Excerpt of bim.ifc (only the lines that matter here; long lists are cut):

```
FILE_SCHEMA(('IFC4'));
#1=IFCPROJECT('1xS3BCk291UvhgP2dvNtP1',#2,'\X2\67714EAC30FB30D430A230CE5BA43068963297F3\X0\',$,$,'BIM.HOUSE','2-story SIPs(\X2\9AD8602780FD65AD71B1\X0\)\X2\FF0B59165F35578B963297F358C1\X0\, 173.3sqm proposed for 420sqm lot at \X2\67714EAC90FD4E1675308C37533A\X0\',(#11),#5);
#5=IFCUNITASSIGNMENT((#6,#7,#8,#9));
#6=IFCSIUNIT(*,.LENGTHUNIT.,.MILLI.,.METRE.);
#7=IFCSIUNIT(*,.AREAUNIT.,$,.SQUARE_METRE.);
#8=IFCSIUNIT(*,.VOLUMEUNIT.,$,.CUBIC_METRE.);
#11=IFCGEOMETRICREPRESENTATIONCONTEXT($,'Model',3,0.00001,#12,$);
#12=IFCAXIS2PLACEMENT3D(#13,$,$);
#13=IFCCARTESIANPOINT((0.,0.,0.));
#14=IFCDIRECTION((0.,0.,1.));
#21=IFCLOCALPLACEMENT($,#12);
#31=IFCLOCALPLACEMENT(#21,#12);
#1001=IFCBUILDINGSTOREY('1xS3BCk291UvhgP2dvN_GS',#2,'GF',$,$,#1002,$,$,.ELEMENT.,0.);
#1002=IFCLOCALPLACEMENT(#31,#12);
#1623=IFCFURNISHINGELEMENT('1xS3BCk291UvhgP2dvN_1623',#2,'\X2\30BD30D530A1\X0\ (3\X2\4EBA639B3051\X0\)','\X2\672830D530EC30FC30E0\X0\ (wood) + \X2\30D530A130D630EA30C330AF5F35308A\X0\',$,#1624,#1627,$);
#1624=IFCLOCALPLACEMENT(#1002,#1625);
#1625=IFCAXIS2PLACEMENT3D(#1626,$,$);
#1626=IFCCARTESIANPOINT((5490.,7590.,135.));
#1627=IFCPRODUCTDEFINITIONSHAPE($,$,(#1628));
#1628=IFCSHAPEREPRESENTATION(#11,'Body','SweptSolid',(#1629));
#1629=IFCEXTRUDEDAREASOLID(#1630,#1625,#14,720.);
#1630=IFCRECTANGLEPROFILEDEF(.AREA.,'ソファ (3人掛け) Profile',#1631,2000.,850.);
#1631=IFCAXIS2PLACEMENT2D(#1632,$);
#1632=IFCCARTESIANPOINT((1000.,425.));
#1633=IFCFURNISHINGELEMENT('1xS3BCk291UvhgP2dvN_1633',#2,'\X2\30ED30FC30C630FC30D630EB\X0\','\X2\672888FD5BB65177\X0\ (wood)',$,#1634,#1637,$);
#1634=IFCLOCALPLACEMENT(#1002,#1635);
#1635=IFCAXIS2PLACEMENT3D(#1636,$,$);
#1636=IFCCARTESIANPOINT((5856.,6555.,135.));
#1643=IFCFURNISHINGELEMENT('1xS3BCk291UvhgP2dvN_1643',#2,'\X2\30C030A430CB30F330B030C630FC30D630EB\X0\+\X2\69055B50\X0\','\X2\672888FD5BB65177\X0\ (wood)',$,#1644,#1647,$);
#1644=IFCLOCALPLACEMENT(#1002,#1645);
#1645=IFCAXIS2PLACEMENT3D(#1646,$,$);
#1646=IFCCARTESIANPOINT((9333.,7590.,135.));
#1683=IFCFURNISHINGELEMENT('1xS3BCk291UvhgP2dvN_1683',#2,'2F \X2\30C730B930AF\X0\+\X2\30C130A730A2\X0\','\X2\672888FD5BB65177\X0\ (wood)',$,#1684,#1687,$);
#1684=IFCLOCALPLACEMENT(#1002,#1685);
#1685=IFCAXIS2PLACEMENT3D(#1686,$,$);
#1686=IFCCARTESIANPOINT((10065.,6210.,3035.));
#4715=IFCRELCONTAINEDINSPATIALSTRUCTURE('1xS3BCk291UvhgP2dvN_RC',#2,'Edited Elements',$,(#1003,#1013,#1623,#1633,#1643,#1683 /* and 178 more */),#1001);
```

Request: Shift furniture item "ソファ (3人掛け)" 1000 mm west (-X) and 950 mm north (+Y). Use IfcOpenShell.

```python
import ifcopenshell
import ifcopenshell.api.geometry
import ifcopenshell.util.placement
import ifcopenshell.util.unit

model = ifcopenshell.open("bim.ifc")
unit_scale = ifcopenshell.util.unit.calculate_unit_scale(model)

item = model.by_id(1623)
matrix = ifcopenshell.util.placement.get_local_placement(item.ObjectPlacement)
matrix[0, 3] -= 1 / unit_scale
matrix[1, 3] += 0.95 / unit_scale
ifcopenshell.api.geometry.edit_object_placement(model, product=item, matrix=matrix, is_si=False)

print(ifcopenshell.util.placement.get_local_placement(item.ObjectPlacement).round(3) + 0.0)

model.write("bim-out.ifc")
```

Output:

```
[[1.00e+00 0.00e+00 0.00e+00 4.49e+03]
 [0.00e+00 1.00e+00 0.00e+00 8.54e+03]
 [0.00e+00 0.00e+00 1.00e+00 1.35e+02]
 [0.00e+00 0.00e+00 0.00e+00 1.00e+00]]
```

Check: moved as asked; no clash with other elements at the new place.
